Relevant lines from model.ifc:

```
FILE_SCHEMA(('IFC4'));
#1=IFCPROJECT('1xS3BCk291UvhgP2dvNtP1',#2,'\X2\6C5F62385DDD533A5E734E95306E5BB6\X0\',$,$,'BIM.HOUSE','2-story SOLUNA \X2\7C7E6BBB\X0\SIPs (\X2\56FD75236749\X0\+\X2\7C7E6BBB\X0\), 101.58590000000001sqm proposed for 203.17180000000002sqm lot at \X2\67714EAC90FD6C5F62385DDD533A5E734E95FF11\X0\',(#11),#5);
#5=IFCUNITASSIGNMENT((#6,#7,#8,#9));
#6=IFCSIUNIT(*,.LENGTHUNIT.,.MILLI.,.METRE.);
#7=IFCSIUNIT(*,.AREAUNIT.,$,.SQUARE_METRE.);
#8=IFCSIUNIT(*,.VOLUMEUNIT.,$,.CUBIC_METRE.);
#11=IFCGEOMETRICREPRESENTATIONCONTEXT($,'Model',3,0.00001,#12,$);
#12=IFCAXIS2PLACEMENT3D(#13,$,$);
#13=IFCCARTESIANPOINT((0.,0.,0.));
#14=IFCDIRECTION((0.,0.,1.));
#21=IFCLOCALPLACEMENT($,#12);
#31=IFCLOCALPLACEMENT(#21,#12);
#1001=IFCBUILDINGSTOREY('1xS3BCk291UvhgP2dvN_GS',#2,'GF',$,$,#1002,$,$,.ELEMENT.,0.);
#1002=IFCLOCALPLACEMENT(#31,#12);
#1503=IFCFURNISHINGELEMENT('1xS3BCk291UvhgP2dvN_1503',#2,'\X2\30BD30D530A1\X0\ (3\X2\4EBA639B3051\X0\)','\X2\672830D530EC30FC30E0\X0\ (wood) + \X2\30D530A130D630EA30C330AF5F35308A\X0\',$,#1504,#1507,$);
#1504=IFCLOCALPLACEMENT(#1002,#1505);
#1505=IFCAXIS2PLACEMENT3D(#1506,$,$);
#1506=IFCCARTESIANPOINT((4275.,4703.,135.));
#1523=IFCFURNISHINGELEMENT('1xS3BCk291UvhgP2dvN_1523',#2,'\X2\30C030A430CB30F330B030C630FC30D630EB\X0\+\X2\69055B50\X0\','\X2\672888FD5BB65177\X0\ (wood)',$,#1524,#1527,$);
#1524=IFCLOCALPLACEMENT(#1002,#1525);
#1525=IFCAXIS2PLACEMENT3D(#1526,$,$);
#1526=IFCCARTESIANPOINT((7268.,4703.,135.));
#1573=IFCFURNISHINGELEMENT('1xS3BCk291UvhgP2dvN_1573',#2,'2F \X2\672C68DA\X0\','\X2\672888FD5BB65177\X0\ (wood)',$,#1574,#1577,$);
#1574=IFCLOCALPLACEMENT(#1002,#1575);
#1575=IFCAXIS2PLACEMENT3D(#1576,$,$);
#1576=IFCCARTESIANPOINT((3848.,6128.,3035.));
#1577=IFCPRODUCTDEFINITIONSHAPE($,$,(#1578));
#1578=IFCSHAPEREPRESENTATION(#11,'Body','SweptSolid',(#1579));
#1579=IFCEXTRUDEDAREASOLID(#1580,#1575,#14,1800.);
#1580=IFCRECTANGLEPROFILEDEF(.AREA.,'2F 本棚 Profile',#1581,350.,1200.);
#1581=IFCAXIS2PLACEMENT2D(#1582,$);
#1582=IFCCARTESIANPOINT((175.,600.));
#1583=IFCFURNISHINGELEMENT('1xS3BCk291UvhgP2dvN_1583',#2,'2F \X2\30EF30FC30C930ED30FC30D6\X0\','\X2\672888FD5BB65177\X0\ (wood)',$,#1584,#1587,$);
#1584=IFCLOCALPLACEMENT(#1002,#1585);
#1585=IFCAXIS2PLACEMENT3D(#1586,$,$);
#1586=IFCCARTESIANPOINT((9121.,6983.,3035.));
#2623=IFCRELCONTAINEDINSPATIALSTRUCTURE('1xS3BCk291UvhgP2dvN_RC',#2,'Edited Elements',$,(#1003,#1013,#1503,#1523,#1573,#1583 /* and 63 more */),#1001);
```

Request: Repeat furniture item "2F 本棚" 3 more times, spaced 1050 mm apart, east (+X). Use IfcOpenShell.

```python
import numpy as np
import ifcopenshell
import ifcopenshell.api.geometry
import ifcopenshell.api.root
import ifcopenshell.util.element
import ifcopenshell.util.placement
import ifcopenshell.util.unit

model = ifcopenshell.open("model.ifc")
unit_scale = ifcopenshell.util.unit.calculate_unit_scale(model)


def reuse_history(source, copy):
    """copy_class also copies each property set's owner history, people and application; keep the originals."""
    for rel in copy.IsDefinedBy:
        if rel.is_a("IfcRelDefinesByProperties") and (history := rel.RelatingPropertyDefinition.OwnerHistory):
            rel.RelatingPropertyDefinition.OwnerHistory = source.OwnerHistory
            ifcopenshell.util.element.remove_deep2(model, history)


source = model.by_id(1573)
base = ifcopenshell.util.placement.get_local_placement(source.ObjectPlacement)
step = np.array([1.0, 0.0, 0.0]) * 1.05 / unit_scale

for i in range(1, 4):
    copy = ifcopenshell.api.root.copy_class(model, product=source)
    copy.Representation = ifcopenshell.util.element.copy_deep(
        model, source.Representation, exclude=["IfcGeometricRepresentationContext", "IfcRepresentationMap"]
    )
    reuse_history(source, copy)
    matrix = base.copy()
    matrix[:3, 3] += i * step
    print("added at", matrix[:3, 3].round(3) + 0.0)
    ifcopenshell.api.geometry.edit_object_placement(model, product=copy, matrix=matrix, is_si=False)

model.write("model_updated.ifc")
```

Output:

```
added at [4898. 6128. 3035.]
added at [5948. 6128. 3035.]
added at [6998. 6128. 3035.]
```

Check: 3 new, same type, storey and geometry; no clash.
